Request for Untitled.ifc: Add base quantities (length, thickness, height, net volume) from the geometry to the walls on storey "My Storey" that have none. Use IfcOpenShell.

First a look at what the model holds.

```python
import ifcopenshell
import ifcopenshell.util.element
import ifcopenshell.util.unit

model = ifcopenshell.open("Untitled.ifc")
print(model.schema)
for unit_type in ("LENGTHUNIT", "AREAUNIT", "VOLUMEUNIT"):
    print(unit_type, ifcopenshell.util.unit.calculate_unit_scale(model, unit_type))
storey = next(s for s in model.by_type("IfcBuildingStorey") if s.Name == "My Storey")
walls = [e for e in ifcopenshell.util.element.get_decomposition(storey) if e.is_a("IfcWall")]
for e in sorted(walls, key=lambda e: e.id()):
    print(e.id(), e.is_a(), e.Name, list(ifcopenshell.util.element.get_psets(e, qtos_only=True)), sep=" | ")
```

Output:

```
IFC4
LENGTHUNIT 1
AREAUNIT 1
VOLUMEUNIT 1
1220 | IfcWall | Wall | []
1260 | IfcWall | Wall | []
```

```python
import ifcopenshell
import ifcopenshell.api.pset
import ifcopenshell.geom
import ifcopenshell.util.element
import ifcopenshell.util.shape
import ifcopenshell.util.unit

model = ifcopenshell.open("Untitled.ifc")
unit_scale = ifcopenshell.util.unit.calculate_unit_scale(model)
volume_scale = ifcopenshell.util.unit.calculate_unit_scale(model, "VOLUMEUNIT")
settings = ifcopenshell.geom.settings()

storey = next(s for s in model.by_type("IfcBuildingStorey") if s.Name == "My Storey")
walls = [e for e in ifcopenshell.util.element.get_decomposition(storey) if e.is_a("IfcWall")]

for e in sorted(walls, key=lambda e: e.id()):
    if ifcopenshell.util.element.get_psets(e, qtos_only=True, should_inherit=False):
        continue
    # Geometry comes back in metres, in the element's own axes.
    shape = ifcopenshell.geom.create_shape(settings, e)
    values = {
        "Length": ifcopenshell.util.shape.get_x(shape.geometry) / unit_scale,
        "Width": ifcopenshell.util.shape.get_y(shape.geometry) / unit_scale,
        "Height": ifcopenshell.util.shape.get_z(shape.geometry) / unit_scale,
        "NetVolume": ifcopenshell.util.shape.get_volume(shape.geometry) / volume_scale,
    }
    qto = ifcopenshell.api.pset.add_qto(model, product=e, name="Qto_WallBaseQuantities")
    ifcopenshell.api.pset.edit_qto(model, qto=qto, properties=values)
    print(e.id(), {k: round(v, 3) for k, v in values.items()})

model.write("Untitled_v2.ifc")
```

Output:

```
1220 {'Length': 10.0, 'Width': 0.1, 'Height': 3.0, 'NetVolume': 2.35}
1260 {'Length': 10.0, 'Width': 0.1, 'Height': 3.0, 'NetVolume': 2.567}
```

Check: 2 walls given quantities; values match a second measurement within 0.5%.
